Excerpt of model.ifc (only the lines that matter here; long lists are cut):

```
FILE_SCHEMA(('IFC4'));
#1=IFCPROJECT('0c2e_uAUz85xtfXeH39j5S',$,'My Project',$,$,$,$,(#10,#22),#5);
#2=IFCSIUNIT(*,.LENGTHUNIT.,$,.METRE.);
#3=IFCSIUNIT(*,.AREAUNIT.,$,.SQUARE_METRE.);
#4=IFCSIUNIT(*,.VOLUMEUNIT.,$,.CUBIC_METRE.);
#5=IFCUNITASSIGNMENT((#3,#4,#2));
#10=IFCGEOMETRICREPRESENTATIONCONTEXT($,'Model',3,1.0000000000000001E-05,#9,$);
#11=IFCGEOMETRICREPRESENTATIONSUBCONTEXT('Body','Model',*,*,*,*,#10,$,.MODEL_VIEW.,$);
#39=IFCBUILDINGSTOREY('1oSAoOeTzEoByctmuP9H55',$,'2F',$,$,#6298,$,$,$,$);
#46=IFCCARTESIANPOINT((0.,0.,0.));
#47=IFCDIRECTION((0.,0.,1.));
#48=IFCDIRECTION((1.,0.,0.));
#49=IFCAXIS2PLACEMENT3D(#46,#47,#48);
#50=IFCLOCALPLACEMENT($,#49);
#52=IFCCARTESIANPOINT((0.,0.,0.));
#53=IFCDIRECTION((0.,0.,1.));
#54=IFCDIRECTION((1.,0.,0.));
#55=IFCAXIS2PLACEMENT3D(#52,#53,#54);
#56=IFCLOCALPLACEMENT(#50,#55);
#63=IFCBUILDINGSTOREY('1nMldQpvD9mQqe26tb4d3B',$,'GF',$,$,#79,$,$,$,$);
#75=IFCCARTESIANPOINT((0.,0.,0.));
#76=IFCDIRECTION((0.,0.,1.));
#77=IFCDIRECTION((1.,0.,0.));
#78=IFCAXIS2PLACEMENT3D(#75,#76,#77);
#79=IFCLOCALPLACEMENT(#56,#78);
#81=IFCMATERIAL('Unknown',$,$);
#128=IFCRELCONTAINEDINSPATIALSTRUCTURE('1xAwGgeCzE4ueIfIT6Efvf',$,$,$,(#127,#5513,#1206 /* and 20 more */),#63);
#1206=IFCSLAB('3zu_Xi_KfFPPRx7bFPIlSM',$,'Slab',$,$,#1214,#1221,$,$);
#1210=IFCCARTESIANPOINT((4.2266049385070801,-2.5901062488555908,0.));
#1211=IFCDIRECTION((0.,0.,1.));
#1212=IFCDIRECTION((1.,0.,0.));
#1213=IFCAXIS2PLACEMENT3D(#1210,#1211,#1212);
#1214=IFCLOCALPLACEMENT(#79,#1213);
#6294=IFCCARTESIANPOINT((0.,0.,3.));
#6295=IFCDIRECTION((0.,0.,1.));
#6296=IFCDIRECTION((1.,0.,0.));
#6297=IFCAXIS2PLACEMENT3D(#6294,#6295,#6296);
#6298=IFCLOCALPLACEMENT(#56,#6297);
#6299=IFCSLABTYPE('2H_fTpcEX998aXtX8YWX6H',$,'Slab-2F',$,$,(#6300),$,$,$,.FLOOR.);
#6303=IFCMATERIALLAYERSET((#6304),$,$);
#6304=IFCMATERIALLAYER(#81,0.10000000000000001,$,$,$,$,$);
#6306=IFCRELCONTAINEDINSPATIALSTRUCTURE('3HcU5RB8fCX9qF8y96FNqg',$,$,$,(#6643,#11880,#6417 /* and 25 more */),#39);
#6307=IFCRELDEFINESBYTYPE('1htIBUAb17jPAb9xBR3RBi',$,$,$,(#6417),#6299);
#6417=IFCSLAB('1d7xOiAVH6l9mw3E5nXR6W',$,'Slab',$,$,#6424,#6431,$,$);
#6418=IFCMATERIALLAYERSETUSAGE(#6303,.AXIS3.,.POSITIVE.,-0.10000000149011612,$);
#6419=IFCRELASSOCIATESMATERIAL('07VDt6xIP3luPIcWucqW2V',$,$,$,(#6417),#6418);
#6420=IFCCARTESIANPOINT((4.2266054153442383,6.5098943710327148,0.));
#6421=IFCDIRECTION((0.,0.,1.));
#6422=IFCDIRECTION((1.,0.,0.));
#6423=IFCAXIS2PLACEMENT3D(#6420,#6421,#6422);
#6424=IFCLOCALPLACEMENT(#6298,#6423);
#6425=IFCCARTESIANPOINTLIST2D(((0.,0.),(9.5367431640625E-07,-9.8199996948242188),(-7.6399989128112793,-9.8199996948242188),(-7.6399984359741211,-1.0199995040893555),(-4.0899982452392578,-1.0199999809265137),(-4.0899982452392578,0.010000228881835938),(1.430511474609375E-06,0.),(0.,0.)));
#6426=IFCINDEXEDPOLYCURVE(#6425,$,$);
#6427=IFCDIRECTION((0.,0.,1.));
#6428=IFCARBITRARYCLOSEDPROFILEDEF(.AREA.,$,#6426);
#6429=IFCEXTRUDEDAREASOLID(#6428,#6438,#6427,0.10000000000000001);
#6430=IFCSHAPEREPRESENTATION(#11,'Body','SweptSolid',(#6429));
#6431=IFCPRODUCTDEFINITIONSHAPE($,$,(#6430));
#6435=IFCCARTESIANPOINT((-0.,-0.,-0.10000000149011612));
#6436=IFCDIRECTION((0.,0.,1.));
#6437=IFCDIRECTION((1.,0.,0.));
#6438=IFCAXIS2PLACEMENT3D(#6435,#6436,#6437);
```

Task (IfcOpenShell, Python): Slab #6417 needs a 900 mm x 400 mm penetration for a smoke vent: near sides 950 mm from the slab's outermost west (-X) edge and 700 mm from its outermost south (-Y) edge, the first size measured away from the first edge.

```python
import numpy as np
import ifcopenshell
import ifcopenshell.api.feature
import ifcopenshell.api.geometry
import ifcopenshell.api.root
import ifcopenshell.geom
import ifcopenshell.util.placement
import ifcopenshell.util.representation
import ifcopenshell.util.shape
import ifcopenshell.util.unit

model = ifcopenshell.open("model.ifc")
unit_scale = ifcopenshell.util.unit.calculate_unit_scale(model)
settings = ifcopenshell.geom.settings()


def volume(element):
    """Net volume in cubic metres, openings subtracted."""
    shape = ifcopenshell.geom.create_shape(settings, element)
    return ifcopenshell.util.shape.get_volume(shape.geometry)


slab = model.by_guid("1d7xOiAVH6l9mw3E5nXR6W")
before = volume(slab)

# Extent in the slab's own axes, in metres. The edges named are its -X and -Y sides.
slab_shape = ifcopenshell.geom.create_shape(settings, slab)
vertices = ifcopenshell.util.shape.get_vertices(slab_shape.geometry)
x_min, y_min, bottom = vertices.min(axis=0)
top = vertices[:, 2].max()

opening = ifcopenshell.api.root.create_entity(model, ifc_class="IfcOpeningElement", name="Smoke vent opening", predefined_type="OPENING")
context = ifcopenshell.util.representation.get_context(model, "Model", "Body", "MODEL_VIEW")
width, depth = 0.9, 0.4
outline = [(0.0, 0.0), (width, 0.0), (width, depth), (0.0, depth), (0.0, 0.0)]
# Overshoot both faces by 50 mm so the cut is clean.
shape = ifcopenshell.api.geometry.add_slab_representation(
    model, context=context, depth=top - bottom + 0.1, polyline=outline
)
ifcopenshell.api.geometry.assign_representation(model, product=opening, representation=shape)

matrix = ifcopenshell.util.placement.get_local_placement(slab.ObjectPlacement)
matrix[:, 3] = matrix @ np.append(np.array([x_min + 0.95, y_min + 0.7, bottom - 0.05]) / unit_scale, 1.0)
ifcopenshell.api.geometry.edit_object_placement(model, product=opening, matrix=matrix, is_si=False)
ifcopenshell.api.feature.add_feature(model, feature=opening, element=slab)

after = volume(slab)

print(f"slab volume {before:.3f} -> {after:.3f} m3")

model.write("model_edited.ifc")
```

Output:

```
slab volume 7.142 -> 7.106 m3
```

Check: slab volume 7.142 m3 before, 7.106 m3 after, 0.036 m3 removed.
